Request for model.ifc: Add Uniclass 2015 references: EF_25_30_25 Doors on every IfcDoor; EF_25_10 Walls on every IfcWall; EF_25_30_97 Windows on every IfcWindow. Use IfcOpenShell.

First a look at what the model holds.

```python
import ifcopenshell

model = ifcopenshell.open("model.ifc")
print(model.schema)
print("classifications:", [c.Name for c in model.by_type("IfcClassification")])
for ifc_class in ("IfcDoor", "IfcRoof", "IfcStair", "IfcWall", "IfcWindow"):
    print(ifc_class, len(model.by_type(ifc_class)))
```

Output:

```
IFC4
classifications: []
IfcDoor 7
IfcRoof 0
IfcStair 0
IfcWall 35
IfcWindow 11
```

```python
import ifcopenshell
import ifcopenshell.api.classification

model = ifcopenshell.open("model.ifc")

system = ifcopenshell.api.classification.add_classification(model, classification="Uniclass 2015")

codes = {
    "IfcDoor": ("EF_25_30_25", "Doors"),
    "IfcWall": ("EF_25_10", "Walls"),
    "IfcWindow": ("EF_25_30_97", "Windows"),
}
for ifc_class, (code, name) in codes.items():
    products = model.by_type(ifc_class)
    ifcopenshell.api.classification.add_reference(
        model, products=products, classification=system, identification=code, name=name
    )
    print(code, len(products))

model.write("model_edited.ifc")
```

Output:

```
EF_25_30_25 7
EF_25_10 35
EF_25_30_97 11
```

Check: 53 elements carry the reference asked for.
